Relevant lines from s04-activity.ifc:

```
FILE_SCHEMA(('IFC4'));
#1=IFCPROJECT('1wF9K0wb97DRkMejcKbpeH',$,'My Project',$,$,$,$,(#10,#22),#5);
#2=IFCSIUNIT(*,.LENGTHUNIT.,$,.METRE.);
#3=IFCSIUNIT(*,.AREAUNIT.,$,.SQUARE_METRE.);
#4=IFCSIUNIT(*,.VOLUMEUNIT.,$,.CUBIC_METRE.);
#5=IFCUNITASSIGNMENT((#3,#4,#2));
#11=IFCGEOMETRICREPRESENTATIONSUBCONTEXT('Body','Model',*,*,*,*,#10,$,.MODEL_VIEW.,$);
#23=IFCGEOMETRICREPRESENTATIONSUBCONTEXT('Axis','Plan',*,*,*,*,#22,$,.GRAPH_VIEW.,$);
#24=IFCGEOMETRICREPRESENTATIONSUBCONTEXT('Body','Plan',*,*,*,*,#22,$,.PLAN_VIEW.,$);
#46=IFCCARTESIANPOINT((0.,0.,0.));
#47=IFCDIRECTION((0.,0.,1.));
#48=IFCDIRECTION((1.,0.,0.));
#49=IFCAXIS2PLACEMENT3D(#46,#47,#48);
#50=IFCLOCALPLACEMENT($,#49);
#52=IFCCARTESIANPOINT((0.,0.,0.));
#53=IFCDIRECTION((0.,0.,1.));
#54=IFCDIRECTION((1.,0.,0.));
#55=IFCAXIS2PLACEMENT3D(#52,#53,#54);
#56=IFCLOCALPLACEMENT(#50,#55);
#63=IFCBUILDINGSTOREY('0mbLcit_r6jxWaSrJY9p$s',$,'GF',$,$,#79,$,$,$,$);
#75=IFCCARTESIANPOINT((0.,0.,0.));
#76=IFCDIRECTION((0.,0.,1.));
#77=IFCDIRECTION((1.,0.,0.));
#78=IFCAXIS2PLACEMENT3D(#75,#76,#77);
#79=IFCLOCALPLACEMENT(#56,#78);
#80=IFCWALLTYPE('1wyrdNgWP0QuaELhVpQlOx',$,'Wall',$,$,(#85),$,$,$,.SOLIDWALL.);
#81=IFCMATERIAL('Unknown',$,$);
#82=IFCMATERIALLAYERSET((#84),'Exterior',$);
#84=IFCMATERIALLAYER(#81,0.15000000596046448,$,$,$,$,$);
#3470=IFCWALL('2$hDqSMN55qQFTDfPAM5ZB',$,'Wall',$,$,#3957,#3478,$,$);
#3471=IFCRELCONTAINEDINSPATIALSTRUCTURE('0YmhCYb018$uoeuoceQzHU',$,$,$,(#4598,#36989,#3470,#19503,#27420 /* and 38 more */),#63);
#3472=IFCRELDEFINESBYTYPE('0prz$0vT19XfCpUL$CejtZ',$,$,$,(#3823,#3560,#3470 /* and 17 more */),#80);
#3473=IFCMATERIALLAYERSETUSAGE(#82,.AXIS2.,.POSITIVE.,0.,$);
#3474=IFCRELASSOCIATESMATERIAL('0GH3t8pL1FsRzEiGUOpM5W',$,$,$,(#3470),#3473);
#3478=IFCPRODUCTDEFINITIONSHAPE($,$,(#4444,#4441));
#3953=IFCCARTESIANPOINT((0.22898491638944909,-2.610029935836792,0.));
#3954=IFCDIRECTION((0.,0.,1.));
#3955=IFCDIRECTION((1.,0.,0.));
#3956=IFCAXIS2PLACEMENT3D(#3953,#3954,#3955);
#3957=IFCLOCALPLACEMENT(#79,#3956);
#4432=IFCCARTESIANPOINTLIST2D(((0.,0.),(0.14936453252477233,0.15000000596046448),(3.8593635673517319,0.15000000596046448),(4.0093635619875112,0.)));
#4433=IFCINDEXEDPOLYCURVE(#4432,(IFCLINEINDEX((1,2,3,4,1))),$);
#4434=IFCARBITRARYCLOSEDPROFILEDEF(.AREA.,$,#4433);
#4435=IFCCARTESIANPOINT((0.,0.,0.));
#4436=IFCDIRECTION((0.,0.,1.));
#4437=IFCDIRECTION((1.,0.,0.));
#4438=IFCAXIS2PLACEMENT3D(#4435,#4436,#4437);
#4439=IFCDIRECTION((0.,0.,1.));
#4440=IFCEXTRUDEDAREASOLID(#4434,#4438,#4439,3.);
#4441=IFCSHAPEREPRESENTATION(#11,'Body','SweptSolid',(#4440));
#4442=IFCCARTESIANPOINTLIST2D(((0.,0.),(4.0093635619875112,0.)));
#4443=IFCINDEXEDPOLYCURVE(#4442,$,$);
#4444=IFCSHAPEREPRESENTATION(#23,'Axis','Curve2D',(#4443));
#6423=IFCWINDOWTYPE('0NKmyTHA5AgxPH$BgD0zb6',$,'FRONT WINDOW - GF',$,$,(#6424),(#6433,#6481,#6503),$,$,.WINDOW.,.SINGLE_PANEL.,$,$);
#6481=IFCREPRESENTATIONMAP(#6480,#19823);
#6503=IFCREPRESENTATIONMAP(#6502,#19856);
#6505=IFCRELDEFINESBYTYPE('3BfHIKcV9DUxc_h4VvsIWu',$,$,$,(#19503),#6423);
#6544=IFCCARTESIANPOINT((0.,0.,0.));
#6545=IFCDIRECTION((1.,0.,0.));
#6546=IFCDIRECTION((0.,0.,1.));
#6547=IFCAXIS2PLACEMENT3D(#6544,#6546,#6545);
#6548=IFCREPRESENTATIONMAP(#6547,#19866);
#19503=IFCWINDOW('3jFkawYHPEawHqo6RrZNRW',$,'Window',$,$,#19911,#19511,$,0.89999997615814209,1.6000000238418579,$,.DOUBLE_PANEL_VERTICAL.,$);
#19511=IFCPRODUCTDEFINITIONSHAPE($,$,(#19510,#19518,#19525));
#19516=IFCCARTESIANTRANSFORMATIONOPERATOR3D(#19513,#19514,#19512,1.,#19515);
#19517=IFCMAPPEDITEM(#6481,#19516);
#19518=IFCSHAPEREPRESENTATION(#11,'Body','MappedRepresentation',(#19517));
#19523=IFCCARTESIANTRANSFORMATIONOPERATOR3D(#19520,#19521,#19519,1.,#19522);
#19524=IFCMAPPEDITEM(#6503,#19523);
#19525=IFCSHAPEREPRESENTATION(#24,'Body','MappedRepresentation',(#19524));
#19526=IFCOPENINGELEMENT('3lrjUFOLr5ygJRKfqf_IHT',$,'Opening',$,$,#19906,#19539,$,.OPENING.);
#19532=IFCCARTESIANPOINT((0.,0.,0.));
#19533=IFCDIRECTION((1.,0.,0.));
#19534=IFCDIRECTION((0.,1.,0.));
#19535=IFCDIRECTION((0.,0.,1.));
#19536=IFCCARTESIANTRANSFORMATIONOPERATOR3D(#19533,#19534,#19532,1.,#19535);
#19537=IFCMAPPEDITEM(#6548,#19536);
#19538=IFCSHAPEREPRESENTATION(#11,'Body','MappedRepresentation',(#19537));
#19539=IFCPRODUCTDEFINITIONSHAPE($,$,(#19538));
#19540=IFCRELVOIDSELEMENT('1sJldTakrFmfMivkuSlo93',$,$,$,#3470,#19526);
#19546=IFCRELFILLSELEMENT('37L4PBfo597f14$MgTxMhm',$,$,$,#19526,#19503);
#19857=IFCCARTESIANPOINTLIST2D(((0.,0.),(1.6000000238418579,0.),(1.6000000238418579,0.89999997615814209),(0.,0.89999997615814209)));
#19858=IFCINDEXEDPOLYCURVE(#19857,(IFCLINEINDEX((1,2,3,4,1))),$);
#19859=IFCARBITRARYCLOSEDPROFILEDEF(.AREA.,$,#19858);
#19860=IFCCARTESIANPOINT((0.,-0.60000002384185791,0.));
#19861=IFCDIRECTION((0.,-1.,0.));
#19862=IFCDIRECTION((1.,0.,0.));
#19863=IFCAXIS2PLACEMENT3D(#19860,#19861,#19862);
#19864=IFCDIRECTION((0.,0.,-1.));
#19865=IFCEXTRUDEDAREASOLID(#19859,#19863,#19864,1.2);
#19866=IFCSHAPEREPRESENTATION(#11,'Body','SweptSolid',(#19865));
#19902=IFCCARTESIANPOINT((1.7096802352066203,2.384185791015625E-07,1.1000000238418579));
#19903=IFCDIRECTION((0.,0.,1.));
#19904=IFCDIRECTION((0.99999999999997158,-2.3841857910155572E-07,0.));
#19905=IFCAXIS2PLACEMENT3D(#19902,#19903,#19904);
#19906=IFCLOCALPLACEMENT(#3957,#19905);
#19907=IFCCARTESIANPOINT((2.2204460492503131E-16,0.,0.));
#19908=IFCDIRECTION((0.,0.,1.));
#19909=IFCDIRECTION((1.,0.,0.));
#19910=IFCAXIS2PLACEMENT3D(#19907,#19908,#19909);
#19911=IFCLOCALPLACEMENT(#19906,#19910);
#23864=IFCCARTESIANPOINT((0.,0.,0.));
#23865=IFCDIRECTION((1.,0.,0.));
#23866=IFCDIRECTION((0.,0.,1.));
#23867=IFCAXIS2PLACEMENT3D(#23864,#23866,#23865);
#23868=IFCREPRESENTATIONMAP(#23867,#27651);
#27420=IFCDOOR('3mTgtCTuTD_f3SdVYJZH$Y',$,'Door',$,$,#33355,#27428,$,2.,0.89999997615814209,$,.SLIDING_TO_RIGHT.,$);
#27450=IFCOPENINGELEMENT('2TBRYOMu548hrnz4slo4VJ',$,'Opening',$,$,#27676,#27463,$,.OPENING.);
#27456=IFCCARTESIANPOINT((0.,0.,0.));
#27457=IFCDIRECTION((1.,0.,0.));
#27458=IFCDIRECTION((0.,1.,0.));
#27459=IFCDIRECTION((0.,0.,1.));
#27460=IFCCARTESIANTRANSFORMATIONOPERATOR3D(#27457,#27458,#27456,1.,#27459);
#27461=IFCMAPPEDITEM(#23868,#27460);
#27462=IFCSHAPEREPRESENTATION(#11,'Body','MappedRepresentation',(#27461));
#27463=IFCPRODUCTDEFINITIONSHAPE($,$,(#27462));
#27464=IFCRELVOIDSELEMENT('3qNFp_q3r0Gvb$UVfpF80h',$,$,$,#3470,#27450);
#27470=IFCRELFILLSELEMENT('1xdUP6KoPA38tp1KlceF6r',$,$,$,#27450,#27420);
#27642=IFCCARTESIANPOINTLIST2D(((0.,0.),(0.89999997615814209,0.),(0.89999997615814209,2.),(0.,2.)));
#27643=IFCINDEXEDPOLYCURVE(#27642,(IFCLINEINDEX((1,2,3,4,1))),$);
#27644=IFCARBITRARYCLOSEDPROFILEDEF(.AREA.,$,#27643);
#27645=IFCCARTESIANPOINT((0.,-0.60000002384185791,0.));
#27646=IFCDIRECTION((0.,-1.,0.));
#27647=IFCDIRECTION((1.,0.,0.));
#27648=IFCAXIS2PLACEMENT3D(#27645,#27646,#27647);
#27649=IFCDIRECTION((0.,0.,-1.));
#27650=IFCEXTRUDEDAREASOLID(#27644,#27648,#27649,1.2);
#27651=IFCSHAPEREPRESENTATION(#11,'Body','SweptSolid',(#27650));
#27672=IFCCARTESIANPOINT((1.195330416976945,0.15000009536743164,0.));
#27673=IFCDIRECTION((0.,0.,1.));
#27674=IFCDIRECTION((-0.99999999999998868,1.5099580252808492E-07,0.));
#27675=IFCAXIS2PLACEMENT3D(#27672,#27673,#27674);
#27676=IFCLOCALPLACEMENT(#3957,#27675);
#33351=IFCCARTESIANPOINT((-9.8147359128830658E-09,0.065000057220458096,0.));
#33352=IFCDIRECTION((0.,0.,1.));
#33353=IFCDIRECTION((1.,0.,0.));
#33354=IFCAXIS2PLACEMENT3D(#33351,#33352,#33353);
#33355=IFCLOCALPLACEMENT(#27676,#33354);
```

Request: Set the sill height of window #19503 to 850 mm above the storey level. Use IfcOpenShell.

```python
import numpy as np
import ifcopenshell
import ifcopenshell.api.geometry
import ifcopenshell.geom
import ifcopenshell.util.element
import ifcopenshell.util.placement
import ifcopenshell.util.shape
import ifcopenshell.util.unit

model = ifcopenshell.open("s04-activity.ifc")
unit_scale = ifcopenshell.util.unit.calculate_unit_scale(model)

window = model.by_id(19503)
opening = window.FillsVoids[0].RelatingOpeningElement
storey = ifcopenshell.util.element.get_container(window, ifc_class="IfcBuildingStorey")
level = ifcopenshell.util.placement.get_local_placement(storey.ObjectPlacement)[2, 3]

# The opening's origin need not be at the sill, so measure its lowest point.
shape = ifcopenshell.geom.create_shape(ifcopenshell.geom.settings(), opening)
bottom = ifcopenshell.util.shape.get_shape_bottom_elevation(shape, shape.geometry) / unit_scale
dz = level + 0.85 / unit_scale - bottom

shift = np.array([0.0, 0.0, dz])
# The window is placed relative to its opening, so it follows when the opening moves.
matrix = ifcopenshell.util.placement.get_local_placement(opening.ObjectPlacement)
matrix[:3, 3] += shift
ifcopenshell.api.geometry.edit_object_placement(
    model, product=opening, matrix=matrix, is_si=False, should_transform_children=True
)

print(f"moved by {dz * unit_scale:+.3f} m")

model.write("s04-activity_updated.ifc")
```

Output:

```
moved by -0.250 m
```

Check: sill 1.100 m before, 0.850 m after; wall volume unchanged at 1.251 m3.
